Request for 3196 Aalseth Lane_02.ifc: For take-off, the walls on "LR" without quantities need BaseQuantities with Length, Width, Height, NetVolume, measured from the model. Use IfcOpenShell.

First a look at what the model holds.

```python
import ifcopenshell
import ifcopenshell.util.element
import ifcopenshell.util.unit

model = ifcopenshell.open("3196 Aalseth Lane_02.ifc")
print(model.schema)
for unit_type in ("LENGTHUNIT", "AREAUNIT", "VOLUMEUNIT"):
    print(unit_type, ifcopenshell.util.unit.calculate_unit_scale(model, unit_type))
storey = next(s for s in model.by_type("IfcBuildingStorey") if s.Name == "LR")
walls = [e for e in ifcopenshell.util.element.get_decomposition(storey) if e.is_a("IfcWall")]
for e in sorted(walls, key=lambda e: e.id()):
    print(e.id(), e.is_a(), e.Name, list(ifcopenshell.util.element.get_psets(e, qtos_only=True)), sep=" | ")
```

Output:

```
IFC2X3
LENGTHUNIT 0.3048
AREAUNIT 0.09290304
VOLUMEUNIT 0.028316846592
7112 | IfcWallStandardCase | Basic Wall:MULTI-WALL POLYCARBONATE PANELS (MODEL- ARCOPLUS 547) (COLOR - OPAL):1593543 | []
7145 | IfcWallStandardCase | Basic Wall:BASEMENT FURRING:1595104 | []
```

```python
import ifcopenshell
import ifcopenshell.api.pset
import ifcopenshell.geom
import ifcopenshell.util.element
import ifcopenshell.util.shape
import ifcopenshell.util.unit

model = ifcopenshell.open("3196 Aalseth Lane_02.ifc")
unit_scale = ifcopenshell.util.unit.calculate_unit_scale(model)
volume_scale = ifcopenshell.util.unit.calculate_unit_scale(model, "VOLUMEUNIT")
settings = ifcopenshell.geom.settings()

storey = next(s for s in model.by_type("IfcBuildingStorey") if s.Name == "LR")
walls = [e for e in ifcopenshell.util.element.get_decomposition(storey) if e.is_a("IfcWall")]

for e in sorted(walls, key=lambda e: e.id()):
    if ifcopenshell.util.element.get_psets(e, qtos_only=True, should_inherit=False):
        continue
    # Geometry comes back in metres, in the element's own axes.
    shape = ifcopenshell.geom.create_shape(settings, e)
    values = {
        "Length": ifcopenshell.util.shape.get_x(shape.geometry) / unit_scale,
        "Width": ifcopenshell.util.shape.get_y(shape.geometry) / unit_scale,
        "Height": ifcopenshell.util.shape.get_z(shape.geometry) / unit_scale,
        "NetVolume": ifcopenshell.util.shape.get_volume(shape.geometry) / volume_scale,
    }
    qto = ifcopenshell.api.pset.add_qto(model, product=e, name="BaseQuantities")
    ifcopenshell.api.pset.edit_qto(model, qto=qto, properties=values)
    print(e.id(), {k: round(v, 3) for k, v in values.items()})

model.write("3196 Aalseth Lane_02-out.ifc")
```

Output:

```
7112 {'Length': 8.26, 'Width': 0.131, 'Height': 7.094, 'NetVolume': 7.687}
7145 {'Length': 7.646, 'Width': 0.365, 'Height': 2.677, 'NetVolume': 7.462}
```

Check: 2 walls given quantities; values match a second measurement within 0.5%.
